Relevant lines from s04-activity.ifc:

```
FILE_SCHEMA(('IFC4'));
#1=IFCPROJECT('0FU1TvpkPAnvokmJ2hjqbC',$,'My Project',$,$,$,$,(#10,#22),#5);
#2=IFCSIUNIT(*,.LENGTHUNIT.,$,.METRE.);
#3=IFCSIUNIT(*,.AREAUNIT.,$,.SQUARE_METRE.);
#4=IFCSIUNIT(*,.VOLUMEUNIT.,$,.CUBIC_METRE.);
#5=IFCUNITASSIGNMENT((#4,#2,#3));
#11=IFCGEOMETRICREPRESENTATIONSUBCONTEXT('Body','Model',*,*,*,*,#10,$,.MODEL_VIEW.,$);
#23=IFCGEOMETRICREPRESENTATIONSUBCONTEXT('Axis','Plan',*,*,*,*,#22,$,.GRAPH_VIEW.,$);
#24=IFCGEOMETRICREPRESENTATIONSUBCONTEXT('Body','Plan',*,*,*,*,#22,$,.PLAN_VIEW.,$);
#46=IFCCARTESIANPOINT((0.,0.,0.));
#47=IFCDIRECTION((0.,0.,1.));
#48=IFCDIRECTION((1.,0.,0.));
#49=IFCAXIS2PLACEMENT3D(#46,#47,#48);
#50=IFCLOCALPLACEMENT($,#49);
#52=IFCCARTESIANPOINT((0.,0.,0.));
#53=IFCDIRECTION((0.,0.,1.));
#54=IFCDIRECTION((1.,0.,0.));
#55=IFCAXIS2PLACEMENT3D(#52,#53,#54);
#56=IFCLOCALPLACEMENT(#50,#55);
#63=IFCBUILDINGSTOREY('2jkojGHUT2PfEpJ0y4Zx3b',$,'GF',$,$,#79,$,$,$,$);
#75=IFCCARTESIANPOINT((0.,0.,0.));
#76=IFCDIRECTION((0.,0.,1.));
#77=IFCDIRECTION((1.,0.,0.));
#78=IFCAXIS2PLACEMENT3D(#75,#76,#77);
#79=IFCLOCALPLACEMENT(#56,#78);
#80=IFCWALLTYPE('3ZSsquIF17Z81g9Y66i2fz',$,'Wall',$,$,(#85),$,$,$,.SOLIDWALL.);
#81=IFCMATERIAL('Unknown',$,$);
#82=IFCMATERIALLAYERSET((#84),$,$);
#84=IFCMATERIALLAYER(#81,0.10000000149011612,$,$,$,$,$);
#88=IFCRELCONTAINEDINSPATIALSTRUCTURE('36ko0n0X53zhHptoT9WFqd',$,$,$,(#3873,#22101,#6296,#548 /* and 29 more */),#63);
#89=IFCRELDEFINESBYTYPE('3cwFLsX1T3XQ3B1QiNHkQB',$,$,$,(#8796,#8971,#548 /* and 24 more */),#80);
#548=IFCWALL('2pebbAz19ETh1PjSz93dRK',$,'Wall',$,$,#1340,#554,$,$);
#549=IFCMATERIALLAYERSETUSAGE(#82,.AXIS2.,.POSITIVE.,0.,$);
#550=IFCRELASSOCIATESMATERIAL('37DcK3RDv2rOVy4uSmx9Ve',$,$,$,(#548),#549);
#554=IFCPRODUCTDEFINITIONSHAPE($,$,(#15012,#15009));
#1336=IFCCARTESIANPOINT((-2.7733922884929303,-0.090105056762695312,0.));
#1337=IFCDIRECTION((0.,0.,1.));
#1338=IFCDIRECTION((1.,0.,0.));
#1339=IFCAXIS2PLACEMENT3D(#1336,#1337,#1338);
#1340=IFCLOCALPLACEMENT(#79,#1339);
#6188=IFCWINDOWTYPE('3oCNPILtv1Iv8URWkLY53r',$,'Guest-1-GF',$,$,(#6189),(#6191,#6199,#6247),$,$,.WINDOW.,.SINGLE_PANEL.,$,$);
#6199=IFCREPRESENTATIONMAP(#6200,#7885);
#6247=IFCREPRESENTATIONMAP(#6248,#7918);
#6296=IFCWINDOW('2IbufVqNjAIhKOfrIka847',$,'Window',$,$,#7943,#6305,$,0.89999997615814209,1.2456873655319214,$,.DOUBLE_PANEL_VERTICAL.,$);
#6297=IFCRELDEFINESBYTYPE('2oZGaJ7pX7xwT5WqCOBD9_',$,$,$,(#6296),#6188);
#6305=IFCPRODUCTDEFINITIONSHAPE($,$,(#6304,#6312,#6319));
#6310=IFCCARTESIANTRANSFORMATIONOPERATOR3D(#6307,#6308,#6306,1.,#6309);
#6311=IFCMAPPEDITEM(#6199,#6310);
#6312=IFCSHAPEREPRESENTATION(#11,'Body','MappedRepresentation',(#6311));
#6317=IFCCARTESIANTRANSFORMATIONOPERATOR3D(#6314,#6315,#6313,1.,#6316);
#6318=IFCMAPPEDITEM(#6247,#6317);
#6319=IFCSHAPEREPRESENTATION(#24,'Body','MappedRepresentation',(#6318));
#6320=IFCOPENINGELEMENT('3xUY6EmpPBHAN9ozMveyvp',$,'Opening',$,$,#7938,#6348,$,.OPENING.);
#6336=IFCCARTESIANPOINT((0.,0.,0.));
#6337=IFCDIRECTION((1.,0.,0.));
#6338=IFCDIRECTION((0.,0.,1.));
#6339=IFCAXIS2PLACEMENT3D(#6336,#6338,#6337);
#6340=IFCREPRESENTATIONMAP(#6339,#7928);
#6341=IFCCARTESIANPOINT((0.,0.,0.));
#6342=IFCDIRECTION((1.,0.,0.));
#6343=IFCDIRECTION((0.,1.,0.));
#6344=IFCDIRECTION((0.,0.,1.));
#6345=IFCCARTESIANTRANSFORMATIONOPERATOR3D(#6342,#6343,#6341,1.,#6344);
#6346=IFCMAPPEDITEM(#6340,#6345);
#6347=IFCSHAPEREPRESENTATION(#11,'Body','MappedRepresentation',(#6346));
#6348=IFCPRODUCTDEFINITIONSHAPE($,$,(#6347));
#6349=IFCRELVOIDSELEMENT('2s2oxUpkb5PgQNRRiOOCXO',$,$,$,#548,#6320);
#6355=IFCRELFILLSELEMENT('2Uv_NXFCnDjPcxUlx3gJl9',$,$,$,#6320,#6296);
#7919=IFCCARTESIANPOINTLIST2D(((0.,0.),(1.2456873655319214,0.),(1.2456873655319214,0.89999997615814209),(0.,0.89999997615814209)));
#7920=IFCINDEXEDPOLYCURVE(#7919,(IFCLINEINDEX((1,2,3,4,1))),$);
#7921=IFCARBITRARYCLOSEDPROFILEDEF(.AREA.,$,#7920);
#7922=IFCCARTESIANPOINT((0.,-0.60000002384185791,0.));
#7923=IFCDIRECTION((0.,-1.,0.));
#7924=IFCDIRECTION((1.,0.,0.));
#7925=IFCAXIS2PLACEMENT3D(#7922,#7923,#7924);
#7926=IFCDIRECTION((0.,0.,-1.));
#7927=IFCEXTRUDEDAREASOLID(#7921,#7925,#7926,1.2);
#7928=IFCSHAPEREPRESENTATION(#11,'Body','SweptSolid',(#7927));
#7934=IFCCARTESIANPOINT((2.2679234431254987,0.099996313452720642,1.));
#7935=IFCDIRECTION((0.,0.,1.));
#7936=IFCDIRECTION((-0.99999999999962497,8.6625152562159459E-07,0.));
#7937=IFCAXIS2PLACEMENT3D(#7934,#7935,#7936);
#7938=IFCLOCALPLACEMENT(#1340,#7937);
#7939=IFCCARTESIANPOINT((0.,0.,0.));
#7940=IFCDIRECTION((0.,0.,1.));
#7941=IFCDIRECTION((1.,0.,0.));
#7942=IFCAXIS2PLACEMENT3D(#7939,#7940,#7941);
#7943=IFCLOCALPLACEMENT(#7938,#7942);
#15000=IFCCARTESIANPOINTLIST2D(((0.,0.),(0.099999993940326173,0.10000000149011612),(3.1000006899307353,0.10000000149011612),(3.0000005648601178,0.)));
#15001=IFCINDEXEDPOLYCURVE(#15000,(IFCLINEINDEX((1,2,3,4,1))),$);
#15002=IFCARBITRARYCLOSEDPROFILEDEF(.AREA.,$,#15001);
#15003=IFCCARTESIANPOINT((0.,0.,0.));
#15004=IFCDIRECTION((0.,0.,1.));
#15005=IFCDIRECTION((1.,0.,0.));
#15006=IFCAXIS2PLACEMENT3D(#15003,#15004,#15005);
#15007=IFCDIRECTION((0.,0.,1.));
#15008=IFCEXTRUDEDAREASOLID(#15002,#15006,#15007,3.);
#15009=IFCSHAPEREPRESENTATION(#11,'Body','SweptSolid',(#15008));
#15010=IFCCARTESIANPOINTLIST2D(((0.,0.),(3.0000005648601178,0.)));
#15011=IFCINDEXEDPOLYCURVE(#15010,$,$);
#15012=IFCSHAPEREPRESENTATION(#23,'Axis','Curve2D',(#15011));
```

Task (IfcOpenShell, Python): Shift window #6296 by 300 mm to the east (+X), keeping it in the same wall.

```python
import ifcopenshell
import ifcopenshell.api.geometry
import ifcopenshell.util.placement

model = ifcopenshell.open("s04-activity.ifc")

window = model.by_guid("2IbufVqNjAIhKOfrIka847")
opening = window.FillsVoids[0].RelatingOpeningElement
wall = opening.VoidsElements[0].RelatingBuildingElement

wall_matrix = ifcopenshell.util.placement.get_local_placement(wall.ObjectPlacement)
shift = wall_matrix[:3, 0] * 0.3
before = ifcopenshell.util.placement.get_local_placement(window.ObjectPlacement)[:3, 3].copy()

# The window is placed relative to its opening, so it follows when the opening moves.
matrix = ifcopenshell.util.placement.get_local_placement(opening.ObjectPlacement)
matrix[:3, 3] += shift
ifcopenshell.api.geometry.edit_object_placement(
    model, product=opening, matrix=matrix, is_si=False, should_transform_children=True
)

after = ifcopenshell.util.placement.get_local_placement(window.ObjectPlacement)[:3, 3]
print("window moved by", (after - before).round(3) + 0.0)

model.write("s04-activity_rev.ifc")
```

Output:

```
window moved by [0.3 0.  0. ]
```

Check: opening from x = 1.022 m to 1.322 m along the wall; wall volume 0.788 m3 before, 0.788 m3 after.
